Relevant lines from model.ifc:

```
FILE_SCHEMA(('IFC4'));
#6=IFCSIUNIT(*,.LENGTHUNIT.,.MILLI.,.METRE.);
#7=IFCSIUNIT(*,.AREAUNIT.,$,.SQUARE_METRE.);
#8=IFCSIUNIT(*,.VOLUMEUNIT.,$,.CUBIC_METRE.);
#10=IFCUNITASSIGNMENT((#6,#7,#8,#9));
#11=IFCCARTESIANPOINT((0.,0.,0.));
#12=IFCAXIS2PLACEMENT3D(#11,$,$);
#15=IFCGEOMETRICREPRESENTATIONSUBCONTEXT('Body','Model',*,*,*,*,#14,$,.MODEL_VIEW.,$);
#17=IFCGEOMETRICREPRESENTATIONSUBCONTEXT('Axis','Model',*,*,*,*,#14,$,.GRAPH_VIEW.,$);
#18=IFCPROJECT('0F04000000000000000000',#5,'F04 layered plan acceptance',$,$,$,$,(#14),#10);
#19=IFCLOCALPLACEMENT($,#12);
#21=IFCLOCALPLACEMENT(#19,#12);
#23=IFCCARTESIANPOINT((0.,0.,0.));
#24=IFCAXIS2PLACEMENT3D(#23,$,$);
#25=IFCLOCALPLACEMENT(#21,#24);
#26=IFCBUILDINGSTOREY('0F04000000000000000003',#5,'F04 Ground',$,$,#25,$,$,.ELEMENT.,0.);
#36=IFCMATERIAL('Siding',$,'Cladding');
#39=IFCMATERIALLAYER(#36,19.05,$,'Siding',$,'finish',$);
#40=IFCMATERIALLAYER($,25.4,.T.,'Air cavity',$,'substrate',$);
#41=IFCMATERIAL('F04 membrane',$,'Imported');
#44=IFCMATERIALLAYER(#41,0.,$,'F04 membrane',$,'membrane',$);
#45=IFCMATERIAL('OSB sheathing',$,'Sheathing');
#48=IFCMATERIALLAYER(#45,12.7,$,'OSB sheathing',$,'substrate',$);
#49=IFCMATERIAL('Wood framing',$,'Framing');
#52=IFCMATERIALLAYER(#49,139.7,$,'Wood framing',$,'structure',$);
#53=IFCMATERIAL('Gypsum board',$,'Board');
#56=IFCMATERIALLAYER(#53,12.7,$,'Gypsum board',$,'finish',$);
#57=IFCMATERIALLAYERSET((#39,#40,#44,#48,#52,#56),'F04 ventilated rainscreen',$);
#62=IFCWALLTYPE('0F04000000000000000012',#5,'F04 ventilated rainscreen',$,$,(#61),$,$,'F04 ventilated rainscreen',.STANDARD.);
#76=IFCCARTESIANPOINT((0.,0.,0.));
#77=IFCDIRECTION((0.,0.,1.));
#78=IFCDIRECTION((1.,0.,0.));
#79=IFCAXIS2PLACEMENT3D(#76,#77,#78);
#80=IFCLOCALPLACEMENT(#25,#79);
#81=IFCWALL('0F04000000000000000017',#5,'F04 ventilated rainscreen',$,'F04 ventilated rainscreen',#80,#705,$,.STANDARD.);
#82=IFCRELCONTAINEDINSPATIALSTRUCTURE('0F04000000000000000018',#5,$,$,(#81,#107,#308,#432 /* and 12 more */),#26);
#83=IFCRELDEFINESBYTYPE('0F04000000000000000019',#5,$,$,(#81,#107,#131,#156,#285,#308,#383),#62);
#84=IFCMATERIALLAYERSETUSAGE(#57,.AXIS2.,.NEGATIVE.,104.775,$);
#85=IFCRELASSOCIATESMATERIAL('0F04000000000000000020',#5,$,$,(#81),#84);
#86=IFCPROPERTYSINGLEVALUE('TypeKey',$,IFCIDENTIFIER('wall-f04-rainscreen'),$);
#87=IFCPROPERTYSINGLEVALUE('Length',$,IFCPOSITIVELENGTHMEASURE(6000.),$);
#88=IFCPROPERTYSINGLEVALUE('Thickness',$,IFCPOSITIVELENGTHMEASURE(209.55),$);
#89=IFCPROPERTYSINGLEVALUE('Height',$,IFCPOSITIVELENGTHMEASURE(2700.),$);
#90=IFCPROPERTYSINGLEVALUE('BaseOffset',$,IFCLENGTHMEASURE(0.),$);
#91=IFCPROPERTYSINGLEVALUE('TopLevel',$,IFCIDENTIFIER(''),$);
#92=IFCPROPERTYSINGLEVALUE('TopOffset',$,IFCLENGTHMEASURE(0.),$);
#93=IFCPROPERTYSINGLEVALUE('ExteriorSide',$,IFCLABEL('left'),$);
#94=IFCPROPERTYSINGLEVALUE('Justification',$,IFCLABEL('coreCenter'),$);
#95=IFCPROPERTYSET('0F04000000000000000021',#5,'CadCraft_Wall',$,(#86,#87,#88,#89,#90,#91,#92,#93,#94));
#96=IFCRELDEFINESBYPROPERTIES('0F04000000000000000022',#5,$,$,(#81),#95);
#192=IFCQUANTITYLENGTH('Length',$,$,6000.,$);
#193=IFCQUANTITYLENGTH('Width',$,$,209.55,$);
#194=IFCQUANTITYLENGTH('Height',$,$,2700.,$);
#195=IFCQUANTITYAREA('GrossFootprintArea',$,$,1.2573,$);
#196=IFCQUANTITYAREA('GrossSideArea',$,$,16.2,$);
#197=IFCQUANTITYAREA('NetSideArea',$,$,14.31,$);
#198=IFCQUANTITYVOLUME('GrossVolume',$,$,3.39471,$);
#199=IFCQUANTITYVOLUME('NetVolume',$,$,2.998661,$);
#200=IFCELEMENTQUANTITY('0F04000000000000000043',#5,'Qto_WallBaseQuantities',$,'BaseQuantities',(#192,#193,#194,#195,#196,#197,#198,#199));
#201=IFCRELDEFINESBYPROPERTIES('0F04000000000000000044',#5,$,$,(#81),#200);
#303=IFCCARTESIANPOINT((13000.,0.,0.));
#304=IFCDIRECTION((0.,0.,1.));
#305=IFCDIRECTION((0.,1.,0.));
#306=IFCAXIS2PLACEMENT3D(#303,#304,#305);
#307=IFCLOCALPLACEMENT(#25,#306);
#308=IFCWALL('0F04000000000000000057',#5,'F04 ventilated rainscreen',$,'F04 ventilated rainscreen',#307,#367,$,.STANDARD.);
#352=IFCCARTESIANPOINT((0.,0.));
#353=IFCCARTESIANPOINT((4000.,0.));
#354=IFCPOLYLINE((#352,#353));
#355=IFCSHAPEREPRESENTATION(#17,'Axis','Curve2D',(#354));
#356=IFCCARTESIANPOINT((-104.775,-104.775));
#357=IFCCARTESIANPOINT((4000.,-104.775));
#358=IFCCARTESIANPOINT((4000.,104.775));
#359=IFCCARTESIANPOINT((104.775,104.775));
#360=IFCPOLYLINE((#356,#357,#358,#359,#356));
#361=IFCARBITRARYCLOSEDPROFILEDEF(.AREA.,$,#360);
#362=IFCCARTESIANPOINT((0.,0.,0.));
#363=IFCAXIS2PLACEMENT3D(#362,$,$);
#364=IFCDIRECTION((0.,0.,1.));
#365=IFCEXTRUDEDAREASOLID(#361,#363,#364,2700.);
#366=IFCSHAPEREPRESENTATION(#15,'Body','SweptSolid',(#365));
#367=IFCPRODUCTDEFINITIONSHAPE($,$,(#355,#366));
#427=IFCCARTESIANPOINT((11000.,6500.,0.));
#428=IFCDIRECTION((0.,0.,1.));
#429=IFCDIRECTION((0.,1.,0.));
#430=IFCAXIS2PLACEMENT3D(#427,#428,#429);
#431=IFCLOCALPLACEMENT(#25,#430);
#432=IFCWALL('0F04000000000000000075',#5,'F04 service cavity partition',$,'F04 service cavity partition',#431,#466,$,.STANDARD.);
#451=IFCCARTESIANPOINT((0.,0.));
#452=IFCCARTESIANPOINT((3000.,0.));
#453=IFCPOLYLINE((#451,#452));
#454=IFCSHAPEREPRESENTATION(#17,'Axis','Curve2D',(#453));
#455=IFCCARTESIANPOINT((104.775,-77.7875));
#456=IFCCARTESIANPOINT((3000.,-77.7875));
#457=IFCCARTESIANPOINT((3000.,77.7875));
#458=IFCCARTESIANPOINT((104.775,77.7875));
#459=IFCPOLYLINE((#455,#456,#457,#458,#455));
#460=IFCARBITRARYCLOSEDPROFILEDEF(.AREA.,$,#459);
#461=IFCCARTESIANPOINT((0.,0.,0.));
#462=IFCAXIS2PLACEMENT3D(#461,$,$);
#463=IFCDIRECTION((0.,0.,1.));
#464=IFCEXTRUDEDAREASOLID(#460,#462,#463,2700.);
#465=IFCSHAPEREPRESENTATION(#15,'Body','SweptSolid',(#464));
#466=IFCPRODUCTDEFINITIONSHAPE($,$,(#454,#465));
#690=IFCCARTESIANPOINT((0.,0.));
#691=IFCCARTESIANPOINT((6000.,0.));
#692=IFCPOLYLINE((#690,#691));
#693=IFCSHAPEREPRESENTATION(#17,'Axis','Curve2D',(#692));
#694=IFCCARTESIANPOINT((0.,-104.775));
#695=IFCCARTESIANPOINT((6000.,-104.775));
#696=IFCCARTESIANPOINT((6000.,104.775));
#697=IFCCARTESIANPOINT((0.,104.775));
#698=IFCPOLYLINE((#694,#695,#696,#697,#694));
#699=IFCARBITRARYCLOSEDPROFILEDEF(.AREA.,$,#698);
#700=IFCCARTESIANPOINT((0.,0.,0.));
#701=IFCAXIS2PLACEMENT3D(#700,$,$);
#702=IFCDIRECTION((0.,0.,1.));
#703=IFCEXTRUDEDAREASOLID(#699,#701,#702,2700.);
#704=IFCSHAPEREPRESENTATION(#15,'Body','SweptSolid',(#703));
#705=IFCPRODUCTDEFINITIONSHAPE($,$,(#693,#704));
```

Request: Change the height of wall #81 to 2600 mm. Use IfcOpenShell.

```python
import ifcopenshell
import ifcopenshell.api.pset
import ifcopenshell.geom
import ifcopenshell.util.element
import ifcopenshell.util.representation
import ifcopenshell.util.shape
import ifcopenshell.util.unit

model = ifcopenshell.open("model.ifc")
unit_scale = ifcopenshell.util.unit.calculate_unit_scale(model)
area_scale = ifcopenshell.util.unit.calculate_unit_scale(model, "AREAUNIT")
volume_scale = ifcopenshell.util.unit.calculate_unit_scale(model, "VOLUMEUNIT")
settings = ifcopenshell.geom.settings()


def volume(element):
    """Net volume in cubic metres, openings subtracted."""
    shape = ifcopenshell.geom.create_shape(settings, element)
    return ifcopenshell.util.shape.get_volume(shape.geometry)


wall = model.by_guid("0F04000000000000000017")
before = volume(wall)

body = ifcopenshell.util.representation.get_representation(wall, "Model", "Body")
solid = body.Items[0]
old_height = solid.Depth
solid.Depth = 2.6 / unit_scale
after = volume(wall)
thickness = 0.2096  # wall thickness in metres

# Update the stored height, areas and volumes.
pset = model.by_id(ifcopenshell.util.element.get_pset(wall, "CadCraft_Wall", should_inherit=False)["id"])
ifcopenshell.api.pset.edit_pset(model, pset=pset, properties={
    "Height": model.create_entity("IfcPositiveLengthMeasure", solid.Depth),
})
qto = model.by_id(ifcopenshell.util.element.get_pset(wall, "Qto_WallBaseQuantities", should_inherit=False)["id"])
ifcopenshell.api.pset.edit_qto(model, qto=qto, properties={
    "Height": solid.Depth,
    "GrossSideArea": ifcopenshell.util.element.get_pset(wall, "Qto_WallBaseQuantities", "GrossSideArea") * solid.Depth / old_height,
    "NetSideArea": after / thickness / area_scale,
    "GrossVolume": ifcopenshell.util.element.get_pset(wall, "Qto_WallBaseQuantities", "GrossVolume") * solid.Depth / old_height,
    "NetVolume": after / volume_scale,
})

print(f"height {old_height:g} -> {solid.Depth:g}, volume {before:.3f} -> {after:.3f} m3")

model.write("model-out.ifc")
```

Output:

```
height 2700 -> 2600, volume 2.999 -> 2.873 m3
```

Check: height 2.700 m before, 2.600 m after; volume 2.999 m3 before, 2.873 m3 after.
